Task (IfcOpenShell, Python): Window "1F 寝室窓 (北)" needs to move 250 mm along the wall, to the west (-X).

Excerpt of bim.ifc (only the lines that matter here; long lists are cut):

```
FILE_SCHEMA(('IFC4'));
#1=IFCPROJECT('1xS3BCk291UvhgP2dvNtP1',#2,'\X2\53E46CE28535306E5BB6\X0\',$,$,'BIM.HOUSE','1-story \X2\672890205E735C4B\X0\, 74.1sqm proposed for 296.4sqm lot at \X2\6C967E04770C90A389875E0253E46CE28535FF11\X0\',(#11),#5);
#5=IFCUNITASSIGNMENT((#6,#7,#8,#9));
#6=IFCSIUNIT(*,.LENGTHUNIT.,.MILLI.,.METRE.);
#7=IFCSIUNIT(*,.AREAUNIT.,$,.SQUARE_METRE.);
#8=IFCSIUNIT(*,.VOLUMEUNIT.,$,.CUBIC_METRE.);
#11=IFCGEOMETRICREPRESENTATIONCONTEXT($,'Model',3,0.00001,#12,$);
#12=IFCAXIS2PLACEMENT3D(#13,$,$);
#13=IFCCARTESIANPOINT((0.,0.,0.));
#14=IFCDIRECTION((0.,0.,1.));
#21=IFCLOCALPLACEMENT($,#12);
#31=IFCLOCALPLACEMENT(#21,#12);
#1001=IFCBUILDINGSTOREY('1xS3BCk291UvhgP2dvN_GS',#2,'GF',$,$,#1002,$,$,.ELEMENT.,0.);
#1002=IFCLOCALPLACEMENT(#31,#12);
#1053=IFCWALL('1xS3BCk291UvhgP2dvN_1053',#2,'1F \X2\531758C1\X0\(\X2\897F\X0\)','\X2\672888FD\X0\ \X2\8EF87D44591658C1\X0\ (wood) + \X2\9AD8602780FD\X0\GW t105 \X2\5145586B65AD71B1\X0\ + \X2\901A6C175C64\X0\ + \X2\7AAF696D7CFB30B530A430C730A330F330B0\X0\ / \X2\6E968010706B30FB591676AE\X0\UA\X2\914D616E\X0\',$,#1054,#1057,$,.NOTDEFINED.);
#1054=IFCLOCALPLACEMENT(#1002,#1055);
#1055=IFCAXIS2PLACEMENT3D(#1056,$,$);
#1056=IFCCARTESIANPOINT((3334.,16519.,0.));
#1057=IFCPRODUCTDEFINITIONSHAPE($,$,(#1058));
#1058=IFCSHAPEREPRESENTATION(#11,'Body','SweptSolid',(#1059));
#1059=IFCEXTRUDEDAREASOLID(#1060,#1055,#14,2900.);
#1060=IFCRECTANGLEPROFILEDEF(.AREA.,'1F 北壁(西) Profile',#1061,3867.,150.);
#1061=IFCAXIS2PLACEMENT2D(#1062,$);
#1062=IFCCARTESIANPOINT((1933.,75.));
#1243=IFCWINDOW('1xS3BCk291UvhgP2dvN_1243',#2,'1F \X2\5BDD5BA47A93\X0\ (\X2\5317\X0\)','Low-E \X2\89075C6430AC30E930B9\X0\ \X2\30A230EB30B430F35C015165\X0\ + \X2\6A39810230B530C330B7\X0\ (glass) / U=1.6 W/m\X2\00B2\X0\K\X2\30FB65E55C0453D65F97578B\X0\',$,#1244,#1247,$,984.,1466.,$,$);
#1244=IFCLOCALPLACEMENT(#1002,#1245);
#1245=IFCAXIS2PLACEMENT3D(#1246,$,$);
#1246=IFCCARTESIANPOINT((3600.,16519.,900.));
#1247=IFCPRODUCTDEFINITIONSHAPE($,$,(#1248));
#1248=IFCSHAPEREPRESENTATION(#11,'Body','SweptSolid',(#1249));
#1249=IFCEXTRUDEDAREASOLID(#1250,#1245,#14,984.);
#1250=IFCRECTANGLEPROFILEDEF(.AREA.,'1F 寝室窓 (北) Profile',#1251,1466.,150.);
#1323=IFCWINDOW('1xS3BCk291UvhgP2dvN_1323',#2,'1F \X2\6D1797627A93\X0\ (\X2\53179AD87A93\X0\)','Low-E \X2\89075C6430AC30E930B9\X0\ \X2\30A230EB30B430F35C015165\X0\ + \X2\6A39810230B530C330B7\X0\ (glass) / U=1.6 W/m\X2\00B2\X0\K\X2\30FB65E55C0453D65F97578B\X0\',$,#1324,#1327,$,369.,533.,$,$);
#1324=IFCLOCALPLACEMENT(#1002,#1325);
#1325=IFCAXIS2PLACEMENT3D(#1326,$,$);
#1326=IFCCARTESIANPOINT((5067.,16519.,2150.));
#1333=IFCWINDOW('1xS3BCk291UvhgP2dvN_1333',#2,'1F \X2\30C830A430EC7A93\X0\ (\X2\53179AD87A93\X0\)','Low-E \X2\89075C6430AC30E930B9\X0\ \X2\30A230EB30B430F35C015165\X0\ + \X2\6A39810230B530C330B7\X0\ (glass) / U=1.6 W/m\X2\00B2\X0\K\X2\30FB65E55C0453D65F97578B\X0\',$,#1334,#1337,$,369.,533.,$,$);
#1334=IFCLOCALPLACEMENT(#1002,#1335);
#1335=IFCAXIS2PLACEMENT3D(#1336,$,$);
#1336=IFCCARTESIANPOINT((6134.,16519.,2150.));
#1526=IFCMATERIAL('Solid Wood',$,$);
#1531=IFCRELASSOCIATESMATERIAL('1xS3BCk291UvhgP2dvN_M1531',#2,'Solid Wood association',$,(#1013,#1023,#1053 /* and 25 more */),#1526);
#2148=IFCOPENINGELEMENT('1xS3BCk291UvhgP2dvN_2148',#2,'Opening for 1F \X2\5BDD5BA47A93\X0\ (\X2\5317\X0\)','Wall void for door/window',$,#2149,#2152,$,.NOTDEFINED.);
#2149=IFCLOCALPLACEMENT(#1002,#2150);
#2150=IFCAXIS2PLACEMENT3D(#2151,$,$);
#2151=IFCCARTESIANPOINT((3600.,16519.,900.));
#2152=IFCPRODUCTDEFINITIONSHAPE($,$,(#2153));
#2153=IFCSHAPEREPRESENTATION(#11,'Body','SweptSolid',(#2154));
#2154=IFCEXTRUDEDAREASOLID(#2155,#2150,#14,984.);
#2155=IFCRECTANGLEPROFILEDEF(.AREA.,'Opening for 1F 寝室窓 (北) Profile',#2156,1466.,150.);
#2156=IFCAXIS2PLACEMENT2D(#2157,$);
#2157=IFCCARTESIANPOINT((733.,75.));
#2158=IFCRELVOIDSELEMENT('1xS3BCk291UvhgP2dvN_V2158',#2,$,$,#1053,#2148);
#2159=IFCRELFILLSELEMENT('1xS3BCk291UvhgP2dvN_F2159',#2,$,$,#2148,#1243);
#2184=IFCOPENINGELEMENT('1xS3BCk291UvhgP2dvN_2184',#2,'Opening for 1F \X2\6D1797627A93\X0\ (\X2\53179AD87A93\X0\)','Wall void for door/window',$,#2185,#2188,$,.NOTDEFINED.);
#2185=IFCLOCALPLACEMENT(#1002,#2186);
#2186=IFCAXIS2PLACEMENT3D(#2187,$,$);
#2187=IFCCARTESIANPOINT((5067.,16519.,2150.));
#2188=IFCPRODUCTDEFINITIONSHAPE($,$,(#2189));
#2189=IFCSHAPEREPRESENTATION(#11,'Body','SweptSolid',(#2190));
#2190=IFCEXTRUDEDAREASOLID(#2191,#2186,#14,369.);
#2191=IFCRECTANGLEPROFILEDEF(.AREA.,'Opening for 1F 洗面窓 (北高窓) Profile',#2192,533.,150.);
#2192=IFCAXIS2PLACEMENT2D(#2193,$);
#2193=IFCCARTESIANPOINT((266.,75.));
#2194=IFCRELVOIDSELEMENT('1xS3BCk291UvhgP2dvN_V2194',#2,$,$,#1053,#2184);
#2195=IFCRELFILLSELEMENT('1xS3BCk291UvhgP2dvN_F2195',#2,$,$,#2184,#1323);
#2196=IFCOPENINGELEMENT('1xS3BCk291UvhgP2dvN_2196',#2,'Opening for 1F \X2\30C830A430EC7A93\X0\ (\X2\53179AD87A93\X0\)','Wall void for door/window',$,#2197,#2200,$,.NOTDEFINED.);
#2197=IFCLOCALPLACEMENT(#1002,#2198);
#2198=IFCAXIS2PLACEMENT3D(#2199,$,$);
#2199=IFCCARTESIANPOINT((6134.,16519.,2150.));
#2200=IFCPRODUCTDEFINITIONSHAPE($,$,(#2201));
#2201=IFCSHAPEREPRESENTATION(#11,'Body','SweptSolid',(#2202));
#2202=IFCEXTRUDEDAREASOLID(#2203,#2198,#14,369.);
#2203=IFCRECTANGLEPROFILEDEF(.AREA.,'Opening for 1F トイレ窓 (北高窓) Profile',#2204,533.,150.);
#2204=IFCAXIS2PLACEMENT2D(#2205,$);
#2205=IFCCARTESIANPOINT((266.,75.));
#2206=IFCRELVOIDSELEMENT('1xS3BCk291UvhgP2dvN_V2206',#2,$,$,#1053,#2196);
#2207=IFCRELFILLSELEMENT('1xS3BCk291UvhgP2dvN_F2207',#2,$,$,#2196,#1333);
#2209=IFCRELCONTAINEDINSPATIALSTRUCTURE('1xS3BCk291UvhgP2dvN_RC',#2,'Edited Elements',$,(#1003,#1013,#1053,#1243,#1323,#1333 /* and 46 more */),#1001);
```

```python
import ifcopenshell
import ifcopenshell.api.geometry
import ifcopenshell.util.placement
import ifcopenshell.util.unit

model = ifcopenshell.open("bim.ifc")
unit_scale = ifcopenshell.util.unit.calculate_unit_scale(model)

window = model.by_guid("1xS3BCk291UvhgP2dvN_1243")
opening = window.FillsVoids[0].RelatingOpeningElement
wall = opening.VoidsElements[0].RelatingBuildingElement

wall_matrix = ifcopenshell.util.placement.get_local_placement(wall.ObjectPlacement)
shift = wall_matrix[:3, 0] * -0.25 / unit_scale
before = ifcopenshell.util.placement.get_local_placement(window.ObjectPlacement)[:3, 3].copy()

# The window is not placed relative to its opening, so move both.
for product in (opening, window):
    matrix = ifcopenshell.util.placement.get_local_placement(product.ObjectPlacement)
    matrix[:3, 3] += shift
    ifcopenshell.api.geometry.edit_object_placement(model, product=product, matrix=matrix, is_si=False)

after = ifcopenshell.util.placement.get_local_placement(window.ObjectPlacement)[:3, 3]
print("window moved by", (after - before).round(3) + 0.0)

model.write("bim-out.ifc")
```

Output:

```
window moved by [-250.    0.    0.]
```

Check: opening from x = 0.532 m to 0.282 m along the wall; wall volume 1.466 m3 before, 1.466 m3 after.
